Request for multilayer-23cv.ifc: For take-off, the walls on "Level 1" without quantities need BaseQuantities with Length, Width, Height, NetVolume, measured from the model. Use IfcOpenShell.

First a look at what the model holds.

```python
import ifcopenshell
import ifcopenshell.util.element
import ifcopenshell.util.unit

model = ifcopenshell.open("multilayer-23cv.ifc")
print(model.schema)
for unit_type in ("LENGTHUNIT", "AREAUNIT", "VOLUMEUNIT"):
    print(unit_type, ifcopenshell.util.unit.calculate_unit_scale(model, unit_type))
storey = next(s for s in model.by_type("IfcBuildingStorey") if s.Name == "Level 1")
walls = [e for e in ifcopenshell.util.element.get_decomposition(storey) if e.is_a("IfcWall")]
for e in sorted(walls, key=lambda e: e.id()):
    print(e.id(), e.is_a(), e.Name, list(ifcopenshell.util.element.get_psets(e, qtos_only=True)), sep=" | ")
```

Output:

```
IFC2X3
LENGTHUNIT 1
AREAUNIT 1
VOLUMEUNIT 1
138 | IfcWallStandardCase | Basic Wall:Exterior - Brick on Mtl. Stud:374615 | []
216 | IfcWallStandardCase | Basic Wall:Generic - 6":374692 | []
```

```python
import ifcopenshell
import ifcopenshell.api.pset
import ifcopenshell.geom
import ifcopenshell.util.element
import ifcopenshell.util.shape
import ifcopenshell.util.unit

model = ifcopenshell.open("multilayer-23cv.ifc")
unit_scale = ifcopenshell.util.unit.calculate_unit_scale(model)
volume_scale = ifcopenshell.util.unit.calculate_unit_scale(model, "VOLUMEUNIT")
settings = ifcopenshell.geom.settings()

storey = next(s for s in model.by_type("IfcBuildingStorey") if s.Name == "Level 1")
walls = [e for e in ifcopenshell.util.element.get_decomposition(storey) if e.is_a("IfcWall")]

for e in sorted(walls, key=lambda e: e.id()):
    if ifcopenshell.util.element.get_psets(e, qtos_only=True, should_inherit=False):
        continue
    # Geometry comes back in metres, in the element's own axes.
    shape = ifcopenshell.geom.create_shape(settings, e)
    values = {
        "Length": ifcopenshell.util.shape.get_x(shape.geometry) / unit_scale,
        "Width": ifcopenshell.util.shape.get_y(shape.geometry) / unit_scale,
        "Height": ifcopenshell.util.shape.get_z(shape.geometry) / unit_scale,
        "NetVolume": ifcopenshell.util.shape.get_volume(shape.geometry) / volume_scale,
    }
    qto = ifcopenshell.api.pset.add_qto(model, product=e, name="BaseQuantities")
    ifcopenshell.api.pset.edit_qto(model, qto=qto, properties=values)
    print(e.id(), {k: round(v, 3) for k, v in values.items()})

model.write("multilayer-23cv_edited.ifc")
```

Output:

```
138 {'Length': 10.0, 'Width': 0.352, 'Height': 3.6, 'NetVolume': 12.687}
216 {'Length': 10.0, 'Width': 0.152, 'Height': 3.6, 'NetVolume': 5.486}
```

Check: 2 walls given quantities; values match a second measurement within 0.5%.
